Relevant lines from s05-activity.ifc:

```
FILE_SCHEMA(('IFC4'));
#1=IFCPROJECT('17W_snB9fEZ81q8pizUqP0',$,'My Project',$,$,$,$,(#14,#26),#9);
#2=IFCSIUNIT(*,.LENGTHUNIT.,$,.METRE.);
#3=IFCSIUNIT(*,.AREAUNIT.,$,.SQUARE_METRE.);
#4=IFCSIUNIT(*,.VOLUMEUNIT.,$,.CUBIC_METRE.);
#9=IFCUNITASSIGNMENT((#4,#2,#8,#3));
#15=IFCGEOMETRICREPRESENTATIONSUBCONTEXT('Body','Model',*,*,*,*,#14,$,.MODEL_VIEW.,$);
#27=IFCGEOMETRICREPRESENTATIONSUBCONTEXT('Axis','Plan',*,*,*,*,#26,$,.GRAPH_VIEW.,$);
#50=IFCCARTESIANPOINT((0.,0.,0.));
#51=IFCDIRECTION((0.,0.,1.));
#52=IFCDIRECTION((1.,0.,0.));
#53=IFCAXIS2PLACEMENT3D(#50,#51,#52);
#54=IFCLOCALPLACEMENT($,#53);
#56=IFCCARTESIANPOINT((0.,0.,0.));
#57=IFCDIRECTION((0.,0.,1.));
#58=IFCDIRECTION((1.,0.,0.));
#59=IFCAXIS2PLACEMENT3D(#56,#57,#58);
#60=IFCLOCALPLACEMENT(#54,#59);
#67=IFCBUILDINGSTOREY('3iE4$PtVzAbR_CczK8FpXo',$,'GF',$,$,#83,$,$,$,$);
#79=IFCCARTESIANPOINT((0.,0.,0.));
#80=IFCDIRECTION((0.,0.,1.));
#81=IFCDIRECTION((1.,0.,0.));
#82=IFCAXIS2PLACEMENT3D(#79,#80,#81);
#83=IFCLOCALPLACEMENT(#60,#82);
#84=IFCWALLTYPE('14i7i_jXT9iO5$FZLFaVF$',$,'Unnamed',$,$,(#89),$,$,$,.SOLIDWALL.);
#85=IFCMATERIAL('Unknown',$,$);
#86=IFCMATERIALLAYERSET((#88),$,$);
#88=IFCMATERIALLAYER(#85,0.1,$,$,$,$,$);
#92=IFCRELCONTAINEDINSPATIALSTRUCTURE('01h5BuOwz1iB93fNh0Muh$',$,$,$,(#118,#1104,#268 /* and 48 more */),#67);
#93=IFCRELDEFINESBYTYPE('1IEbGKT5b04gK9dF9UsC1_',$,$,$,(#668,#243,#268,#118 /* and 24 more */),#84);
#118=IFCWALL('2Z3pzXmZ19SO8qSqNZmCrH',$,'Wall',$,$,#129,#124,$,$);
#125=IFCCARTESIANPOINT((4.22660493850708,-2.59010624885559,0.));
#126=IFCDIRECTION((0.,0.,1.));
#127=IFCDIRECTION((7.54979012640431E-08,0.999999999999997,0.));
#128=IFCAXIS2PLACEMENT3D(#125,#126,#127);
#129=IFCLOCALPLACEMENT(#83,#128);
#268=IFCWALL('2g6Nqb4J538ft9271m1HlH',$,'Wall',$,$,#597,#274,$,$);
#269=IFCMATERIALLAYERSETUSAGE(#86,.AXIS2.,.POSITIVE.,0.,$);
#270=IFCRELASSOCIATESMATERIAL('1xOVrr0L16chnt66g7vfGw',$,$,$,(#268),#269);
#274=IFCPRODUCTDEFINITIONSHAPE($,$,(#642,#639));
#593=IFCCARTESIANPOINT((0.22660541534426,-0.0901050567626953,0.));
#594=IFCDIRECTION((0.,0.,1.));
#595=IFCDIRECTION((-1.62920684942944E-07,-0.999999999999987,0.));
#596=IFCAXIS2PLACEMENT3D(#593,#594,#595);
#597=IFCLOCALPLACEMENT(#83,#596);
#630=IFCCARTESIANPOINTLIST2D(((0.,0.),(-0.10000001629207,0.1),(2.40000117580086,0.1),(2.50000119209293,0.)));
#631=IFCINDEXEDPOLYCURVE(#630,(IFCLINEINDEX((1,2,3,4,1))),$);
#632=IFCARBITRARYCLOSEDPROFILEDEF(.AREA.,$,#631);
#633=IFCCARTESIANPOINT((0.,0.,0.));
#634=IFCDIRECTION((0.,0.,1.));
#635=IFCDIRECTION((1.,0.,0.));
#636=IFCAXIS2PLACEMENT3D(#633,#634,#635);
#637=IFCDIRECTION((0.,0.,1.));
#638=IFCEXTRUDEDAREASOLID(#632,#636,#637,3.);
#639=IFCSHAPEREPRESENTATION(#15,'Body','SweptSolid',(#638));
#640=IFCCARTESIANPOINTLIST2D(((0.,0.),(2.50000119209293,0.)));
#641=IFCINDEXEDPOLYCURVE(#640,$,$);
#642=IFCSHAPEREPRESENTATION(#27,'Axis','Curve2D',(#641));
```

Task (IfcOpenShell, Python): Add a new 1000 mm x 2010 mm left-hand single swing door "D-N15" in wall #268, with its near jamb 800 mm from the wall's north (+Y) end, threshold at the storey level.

```python
import numpy as np
import ifcopenshell
import ifcopenshell.api.feature
import ifcopenshell.api.geometry
import ifcopenshell.api.root
import ifcopenshell.api.spatial
import ifcopenshell.geom
import ifcopenshell.util.element
import ifcopenshell.util.placement
import ifcopenshell.util.representation
import ifcopenshell.util.shape
import ifcopenshell.util.unit

model = ifcopenshell.open("s05-activity.ifc")
unit_scale = ifcopenshell.util.unit.calculate_unit_scale(model)
settings = ifcopenshell.geom.settings()


def volume(element):
    """Net volume in cubic metres, openings subtracted."""
    shape = ifcopenshell.geom.create_shape(settings, element)
    return ifcopenshell.util.shape.get_volume(shape.geometry)


wall = model.by_id(268)
storey = ifcopenshell.util.element.get_container(wall, ifc_class="IfcBuildingStorey")
context = ifcopenshell.util.representation.get_context(model, "Model", "Body", "MODEL_VIEW")
before = volume(wall)

width, height, from_end, sill = 1, 2.01, 0.8, 0.0  # metres

# The wall runs along its own X axis, and the end named is its -X end.
wall_shape = ifcopenshell.geom.create_shape(settings, wall)
x, y, z = ifcopenshell.util.shape.get_vertices(wall_shape.geometry).T
start = x.min() + from_end
face, thickness = float(y.min()), float(y.max() - y.min())
wall_matrix = ifcopenshell.util.placement.get_local_placement(wall.ObjectPlacement)
level = ifcopenshell.util.placement.get_local_placement(storey.ObjectPlacement)[2, 3]


def in_wall(x, y):
    """Placement at x, y metres in the wall's axes, at sill height."""
    matrix = wall_matrix.copy()
    matrix[:, 3] = wall_matrix @ np.array([x / unit_scale, y / unit_scale, 0.0, 1.0])
    matrix[2, 3] = level + sill / unit_scale
    return matrix


# Opening: a box that overshoots both wall faces by 50 mm.
opening = ifcopenshell.api.root.create_entity(model, ifc_class="IfcOpeningElement", predefined_type="OPENING")
box = ifcopenshell.api.geometry.add_wall_representation(
    model, context=context, length=width, height=height, thickness=thickness + 0.1
)
ifcopenshell.api.geometry.assign_representation(model, product=opening, representation=box)
ifcopenshell.api.geometry.edit_object_placement(model, product=opening, matrix=in_wall(start, face - 0.05), is_si=False)
ifcopenshell.api.feature.add_feature(model, feature=opening, element=wall)

door = ifcopenshell.api.root.create_entity(model, ifc_class="IfcDoor", name="D-N15", predefined_type="DOOR")
door.OverallWidth, door.OverallHeight = width / unit_scale, height / unit_scale
door.OperationType = "SINGLE_SWING_LEFT"
body = ifcopenshell.api.geometry.add_door_representation(
    model,
    context=context,
    overall_width=door.OverallWidth,
    overall_height=door.OverallHeight,
    operation_type="SINGLE_SWING_LEFT",
    lining_properties={"LiningDepth": thickness / unit_scale, "ThresholdDepth": thickness / unit_scale},
)
ifcopenshell.api.geometry.assign_representation(model, product=door, representation=body)
ifcopenshell.api.spatial.assign_container(model, products=[door], relating_structure=storey)
ifcopenshell.api.feature.add_filling(model, opening=opening, element=door)

# The lining spans the wall, so the door starts at the wall face.
ifcopenshell.api.geometry.edit_object_placement(model, product=door, matrix=in_wall(start, face), is_si=False)

after = volume(wall)

print(f"wall volume {before:.3f} -> {after:.3f} m3")

model.write("s05-activity_edited.ifc")
```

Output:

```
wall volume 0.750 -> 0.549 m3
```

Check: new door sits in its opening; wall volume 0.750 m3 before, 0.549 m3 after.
